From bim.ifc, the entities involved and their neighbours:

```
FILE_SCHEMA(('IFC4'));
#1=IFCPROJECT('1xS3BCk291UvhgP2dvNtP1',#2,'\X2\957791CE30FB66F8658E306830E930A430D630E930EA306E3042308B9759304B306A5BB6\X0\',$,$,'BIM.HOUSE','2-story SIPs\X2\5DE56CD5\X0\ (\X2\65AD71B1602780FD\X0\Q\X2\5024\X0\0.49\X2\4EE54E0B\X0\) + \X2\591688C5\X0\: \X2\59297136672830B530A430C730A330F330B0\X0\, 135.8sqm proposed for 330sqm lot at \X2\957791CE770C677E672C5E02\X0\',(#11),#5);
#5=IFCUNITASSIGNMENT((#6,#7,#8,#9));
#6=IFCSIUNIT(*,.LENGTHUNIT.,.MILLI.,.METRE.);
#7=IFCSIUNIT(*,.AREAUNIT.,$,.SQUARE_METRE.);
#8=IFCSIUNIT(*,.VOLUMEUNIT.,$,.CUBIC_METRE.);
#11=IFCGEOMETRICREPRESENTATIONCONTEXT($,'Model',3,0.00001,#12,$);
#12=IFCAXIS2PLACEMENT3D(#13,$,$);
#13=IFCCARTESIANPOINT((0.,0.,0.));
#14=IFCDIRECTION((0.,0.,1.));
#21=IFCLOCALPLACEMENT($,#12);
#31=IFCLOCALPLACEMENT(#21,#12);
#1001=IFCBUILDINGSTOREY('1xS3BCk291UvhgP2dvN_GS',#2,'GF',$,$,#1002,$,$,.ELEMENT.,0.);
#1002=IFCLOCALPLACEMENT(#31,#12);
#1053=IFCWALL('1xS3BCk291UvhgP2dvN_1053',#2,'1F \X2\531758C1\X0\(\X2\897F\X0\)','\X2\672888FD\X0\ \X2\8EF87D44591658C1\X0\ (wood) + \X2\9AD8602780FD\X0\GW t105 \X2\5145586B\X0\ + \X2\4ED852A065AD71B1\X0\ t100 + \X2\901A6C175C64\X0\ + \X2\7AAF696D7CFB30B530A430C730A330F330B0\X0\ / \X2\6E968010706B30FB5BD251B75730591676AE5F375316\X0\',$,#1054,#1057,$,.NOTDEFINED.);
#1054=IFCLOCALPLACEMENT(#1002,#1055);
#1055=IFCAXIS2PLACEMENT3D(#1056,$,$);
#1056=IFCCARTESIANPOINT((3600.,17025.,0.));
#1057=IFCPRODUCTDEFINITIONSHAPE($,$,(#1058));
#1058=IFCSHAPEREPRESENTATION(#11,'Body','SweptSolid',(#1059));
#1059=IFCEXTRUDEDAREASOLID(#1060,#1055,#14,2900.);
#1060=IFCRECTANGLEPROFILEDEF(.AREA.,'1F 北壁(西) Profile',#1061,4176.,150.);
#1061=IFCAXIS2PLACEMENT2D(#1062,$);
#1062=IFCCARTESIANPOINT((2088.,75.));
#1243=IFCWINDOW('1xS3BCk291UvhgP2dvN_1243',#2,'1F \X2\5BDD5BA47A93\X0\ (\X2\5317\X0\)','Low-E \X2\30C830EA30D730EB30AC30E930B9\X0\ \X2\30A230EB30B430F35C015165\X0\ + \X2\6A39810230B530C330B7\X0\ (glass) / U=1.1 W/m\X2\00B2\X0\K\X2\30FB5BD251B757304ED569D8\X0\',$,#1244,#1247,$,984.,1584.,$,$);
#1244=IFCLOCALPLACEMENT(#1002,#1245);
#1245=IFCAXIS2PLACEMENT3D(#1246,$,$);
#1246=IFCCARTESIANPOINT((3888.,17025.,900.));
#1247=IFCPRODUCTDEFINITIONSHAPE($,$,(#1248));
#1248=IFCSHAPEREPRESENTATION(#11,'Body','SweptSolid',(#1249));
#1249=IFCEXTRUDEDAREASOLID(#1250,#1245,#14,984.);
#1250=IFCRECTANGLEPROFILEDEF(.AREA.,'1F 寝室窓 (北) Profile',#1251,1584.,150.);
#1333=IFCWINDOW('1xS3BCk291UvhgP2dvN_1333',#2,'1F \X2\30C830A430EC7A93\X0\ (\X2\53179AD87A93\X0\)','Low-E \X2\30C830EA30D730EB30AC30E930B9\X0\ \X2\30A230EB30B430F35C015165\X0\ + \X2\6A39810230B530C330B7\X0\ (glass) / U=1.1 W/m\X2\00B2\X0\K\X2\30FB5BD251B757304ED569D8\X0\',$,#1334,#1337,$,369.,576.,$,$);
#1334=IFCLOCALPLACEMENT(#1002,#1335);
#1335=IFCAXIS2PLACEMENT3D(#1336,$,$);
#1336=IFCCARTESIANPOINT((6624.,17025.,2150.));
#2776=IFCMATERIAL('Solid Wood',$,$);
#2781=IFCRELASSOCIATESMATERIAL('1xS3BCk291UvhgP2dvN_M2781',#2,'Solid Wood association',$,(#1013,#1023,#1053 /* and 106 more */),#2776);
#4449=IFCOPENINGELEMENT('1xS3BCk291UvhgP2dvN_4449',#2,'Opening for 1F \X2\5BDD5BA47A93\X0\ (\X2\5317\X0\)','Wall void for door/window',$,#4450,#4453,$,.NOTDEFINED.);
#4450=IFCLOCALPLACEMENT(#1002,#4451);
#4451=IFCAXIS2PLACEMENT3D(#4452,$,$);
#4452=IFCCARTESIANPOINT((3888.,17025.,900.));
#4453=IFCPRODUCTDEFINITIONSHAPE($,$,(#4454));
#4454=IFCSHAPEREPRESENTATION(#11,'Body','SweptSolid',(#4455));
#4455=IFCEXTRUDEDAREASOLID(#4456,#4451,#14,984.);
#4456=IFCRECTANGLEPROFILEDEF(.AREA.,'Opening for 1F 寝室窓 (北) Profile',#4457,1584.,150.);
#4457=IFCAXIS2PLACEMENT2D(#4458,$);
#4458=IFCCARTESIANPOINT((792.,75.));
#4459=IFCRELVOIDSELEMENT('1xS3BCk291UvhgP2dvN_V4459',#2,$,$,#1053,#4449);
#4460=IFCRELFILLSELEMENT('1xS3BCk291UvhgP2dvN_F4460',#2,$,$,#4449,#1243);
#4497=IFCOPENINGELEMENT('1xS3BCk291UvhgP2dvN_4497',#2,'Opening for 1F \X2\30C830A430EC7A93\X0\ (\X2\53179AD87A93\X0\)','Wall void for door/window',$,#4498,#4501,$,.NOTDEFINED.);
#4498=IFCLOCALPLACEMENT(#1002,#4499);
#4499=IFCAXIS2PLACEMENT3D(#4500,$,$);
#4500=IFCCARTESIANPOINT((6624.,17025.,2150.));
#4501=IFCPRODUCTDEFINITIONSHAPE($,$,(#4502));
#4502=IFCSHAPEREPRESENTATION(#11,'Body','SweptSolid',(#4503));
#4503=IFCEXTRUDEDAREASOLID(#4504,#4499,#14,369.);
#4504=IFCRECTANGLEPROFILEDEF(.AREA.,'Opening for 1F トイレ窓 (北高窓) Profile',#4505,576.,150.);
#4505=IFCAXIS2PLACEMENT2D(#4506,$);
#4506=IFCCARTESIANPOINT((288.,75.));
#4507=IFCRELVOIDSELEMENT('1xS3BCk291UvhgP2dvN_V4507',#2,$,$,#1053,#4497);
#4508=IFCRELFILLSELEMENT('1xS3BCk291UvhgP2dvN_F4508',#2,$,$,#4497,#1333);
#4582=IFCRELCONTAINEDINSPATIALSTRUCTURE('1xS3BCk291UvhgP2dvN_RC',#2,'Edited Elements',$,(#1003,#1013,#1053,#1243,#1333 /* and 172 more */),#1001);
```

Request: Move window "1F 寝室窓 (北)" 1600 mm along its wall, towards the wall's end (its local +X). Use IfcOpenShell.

```python
import ifcopenshell
import ifcopenshell.api.geometry
import ifcopenshell.util.placement

model = ifcopenshell.open("bim.ifc")

window = model.by_guid("1xS3BCk291UvhgP2dvN_1243")
opening = window.FillsVoids[0].RelatingOpeningElement
wall = opening.VoidsElements[0].RelatingBuildingElement

wall_matrix = ifcopenshell.util.placement.get_local_placement(wall.ObjectPlacement)
shift = wall_matrix[:3, 0] * 1600.0
before = ifcopenshell.util.placement.get_local_placement(window.ObjectPlacement)[:3, 3].copy()

# The window is not placed relative to its opening, so move both.
for product in (opening, window):
    matrix = ifcopenshell.util.placement.get_local_placement(product.ObjectPlacement)
    matrix[:3, 3] += shift
    ifcopenshell.api.geometry.edit_object_placement(model, product=product, matrix=matrix, is_si=False)

after = ifcopenshell.util.placement.get_local_placement(window.ObjectPlacement)[:3, 3]
print("window moved by", (after - before).round(3) + 0.0)

model.write("bim_edited.ifc")
```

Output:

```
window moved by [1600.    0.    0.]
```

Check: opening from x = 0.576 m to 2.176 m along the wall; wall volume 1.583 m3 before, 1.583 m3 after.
